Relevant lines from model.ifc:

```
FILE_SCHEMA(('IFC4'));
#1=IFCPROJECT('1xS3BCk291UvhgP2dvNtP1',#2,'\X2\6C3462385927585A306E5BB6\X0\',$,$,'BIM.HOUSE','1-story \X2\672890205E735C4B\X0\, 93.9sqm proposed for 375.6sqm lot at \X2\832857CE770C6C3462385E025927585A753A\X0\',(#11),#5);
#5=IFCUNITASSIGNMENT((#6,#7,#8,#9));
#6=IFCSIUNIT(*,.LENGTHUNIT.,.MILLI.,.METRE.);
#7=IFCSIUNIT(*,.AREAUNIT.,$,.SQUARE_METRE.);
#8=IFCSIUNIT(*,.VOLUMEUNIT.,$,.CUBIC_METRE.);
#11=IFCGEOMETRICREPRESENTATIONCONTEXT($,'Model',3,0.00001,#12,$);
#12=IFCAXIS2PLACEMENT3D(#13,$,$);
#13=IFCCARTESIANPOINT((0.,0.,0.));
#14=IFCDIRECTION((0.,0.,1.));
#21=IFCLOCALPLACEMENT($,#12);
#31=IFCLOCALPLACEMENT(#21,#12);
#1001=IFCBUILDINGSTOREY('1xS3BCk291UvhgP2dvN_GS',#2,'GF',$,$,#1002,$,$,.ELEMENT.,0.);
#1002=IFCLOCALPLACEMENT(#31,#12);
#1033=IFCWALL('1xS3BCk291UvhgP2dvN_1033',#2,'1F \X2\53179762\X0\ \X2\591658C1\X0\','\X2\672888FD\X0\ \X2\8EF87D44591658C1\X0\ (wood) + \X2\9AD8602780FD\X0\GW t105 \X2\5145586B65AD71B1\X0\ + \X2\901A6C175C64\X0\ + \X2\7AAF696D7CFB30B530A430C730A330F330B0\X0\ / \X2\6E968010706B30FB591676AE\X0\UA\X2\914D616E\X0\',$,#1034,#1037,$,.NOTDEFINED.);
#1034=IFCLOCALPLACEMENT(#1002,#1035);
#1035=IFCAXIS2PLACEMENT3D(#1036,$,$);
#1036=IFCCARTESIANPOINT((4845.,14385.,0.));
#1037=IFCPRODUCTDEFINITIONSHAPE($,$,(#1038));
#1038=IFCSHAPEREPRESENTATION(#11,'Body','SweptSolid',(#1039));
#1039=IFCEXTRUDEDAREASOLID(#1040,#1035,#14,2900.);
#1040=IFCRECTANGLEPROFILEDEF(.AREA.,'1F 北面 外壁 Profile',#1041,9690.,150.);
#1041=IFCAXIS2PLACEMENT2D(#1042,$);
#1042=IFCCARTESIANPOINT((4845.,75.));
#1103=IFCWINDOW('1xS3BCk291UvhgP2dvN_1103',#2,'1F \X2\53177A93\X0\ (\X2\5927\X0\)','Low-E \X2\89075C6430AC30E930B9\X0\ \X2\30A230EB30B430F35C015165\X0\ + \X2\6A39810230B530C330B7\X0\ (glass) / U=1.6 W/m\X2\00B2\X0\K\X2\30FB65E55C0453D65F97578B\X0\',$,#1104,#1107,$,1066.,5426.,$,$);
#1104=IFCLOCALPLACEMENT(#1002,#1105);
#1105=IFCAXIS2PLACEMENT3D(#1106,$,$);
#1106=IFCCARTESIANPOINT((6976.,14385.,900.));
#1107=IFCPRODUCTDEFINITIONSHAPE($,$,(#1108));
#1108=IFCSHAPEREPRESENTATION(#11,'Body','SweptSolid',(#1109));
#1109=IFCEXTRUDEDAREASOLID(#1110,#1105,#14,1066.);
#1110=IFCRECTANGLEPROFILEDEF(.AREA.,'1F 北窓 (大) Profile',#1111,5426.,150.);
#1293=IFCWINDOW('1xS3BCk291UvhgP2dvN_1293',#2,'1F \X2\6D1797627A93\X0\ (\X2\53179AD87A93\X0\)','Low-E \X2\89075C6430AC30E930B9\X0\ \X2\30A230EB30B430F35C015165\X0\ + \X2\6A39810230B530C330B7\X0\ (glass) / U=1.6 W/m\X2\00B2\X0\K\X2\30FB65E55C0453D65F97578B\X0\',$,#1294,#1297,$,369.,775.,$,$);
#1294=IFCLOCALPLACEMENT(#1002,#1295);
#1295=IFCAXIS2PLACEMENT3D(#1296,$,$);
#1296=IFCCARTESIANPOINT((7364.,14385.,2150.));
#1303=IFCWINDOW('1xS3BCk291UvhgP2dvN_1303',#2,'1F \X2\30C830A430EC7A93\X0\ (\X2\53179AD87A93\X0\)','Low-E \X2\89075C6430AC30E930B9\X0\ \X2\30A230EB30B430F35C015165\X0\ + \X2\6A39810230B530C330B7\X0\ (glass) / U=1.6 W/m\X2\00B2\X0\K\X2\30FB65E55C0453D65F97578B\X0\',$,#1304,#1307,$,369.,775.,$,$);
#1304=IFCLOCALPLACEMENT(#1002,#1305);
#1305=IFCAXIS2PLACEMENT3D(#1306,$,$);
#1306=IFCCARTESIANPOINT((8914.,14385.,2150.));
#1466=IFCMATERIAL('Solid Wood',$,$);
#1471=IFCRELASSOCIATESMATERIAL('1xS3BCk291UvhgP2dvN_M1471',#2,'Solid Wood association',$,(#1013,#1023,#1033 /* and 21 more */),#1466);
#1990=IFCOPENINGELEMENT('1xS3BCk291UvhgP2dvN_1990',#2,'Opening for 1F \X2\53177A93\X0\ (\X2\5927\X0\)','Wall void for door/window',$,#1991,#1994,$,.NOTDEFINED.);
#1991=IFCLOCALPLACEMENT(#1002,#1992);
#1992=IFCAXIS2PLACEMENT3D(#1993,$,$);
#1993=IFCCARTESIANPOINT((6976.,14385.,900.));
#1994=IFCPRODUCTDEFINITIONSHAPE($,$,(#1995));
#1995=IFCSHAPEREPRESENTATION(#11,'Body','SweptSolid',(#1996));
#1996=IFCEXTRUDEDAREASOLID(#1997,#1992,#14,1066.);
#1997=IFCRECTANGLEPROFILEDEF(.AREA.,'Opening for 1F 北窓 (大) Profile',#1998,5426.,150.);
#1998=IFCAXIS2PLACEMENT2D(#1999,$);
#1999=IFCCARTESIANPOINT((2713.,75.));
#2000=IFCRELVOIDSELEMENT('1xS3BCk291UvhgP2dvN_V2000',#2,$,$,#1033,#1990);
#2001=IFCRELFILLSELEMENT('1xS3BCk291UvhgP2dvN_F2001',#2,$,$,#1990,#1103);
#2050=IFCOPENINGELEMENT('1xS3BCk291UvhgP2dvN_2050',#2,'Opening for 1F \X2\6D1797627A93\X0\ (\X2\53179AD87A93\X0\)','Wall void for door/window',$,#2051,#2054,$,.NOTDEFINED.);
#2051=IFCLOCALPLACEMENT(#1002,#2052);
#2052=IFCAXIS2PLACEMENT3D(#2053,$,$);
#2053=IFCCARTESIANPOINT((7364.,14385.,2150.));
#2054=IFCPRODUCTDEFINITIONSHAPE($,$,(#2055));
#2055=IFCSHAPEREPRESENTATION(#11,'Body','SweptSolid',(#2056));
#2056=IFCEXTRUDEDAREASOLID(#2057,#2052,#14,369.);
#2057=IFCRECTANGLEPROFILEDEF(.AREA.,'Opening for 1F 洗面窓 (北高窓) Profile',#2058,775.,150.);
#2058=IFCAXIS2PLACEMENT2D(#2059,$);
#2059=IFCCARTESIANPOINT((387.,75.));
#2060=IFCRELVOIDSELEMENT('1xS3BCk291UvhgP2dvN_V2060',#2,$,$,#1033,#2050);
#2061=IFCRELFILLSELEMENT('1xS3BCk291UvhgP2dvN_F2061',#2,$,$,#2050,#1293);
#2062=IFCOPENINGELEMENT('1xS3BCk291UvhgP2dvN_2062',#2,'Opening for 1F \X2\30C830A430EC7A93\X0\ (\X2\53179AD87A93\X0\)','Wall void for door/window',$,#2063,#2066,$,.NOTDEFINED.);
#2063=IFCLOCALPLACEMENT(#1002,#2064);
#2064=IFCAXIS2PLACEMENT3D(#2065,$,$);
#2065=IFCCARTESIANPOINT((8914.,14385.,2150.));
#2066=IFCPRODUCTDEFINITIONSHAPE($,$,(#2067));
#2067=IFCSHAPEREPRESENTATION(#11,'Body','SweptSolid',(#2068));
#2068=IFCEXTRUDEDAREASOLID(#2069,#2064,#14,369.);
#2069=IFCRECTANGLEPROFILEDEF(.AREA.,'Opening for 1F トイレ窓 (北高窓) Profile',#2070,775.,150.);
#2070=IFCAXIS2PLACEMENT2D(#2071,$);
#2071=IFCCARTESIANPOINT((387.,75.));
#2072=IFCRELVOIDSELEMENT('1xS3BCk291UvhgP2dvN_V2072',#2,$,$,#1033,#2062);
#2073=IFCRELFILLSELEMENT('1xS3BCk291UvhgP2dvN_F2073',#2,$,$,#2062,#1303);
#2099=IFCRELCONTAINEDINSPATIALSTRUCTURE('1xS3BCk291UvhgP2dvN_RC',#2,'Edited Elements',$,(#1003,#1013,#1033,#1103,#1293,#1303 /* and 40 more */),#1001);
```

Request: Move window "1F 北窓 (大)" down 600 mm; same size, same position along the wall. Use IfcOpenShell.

```python
import numpy as np
import ifcopenshell
import ifcopenshell.api.geometry
import ifcopenshell.util.placement
import ifcopenshell.util.unit

model = ifcopenshell.open("model.ifc")
unit_scale = ifcopenshell.util.unit.calculate_unit_scale(model)

window = model.by_guid("1xS3BCk291UvhgP2dvN_1103")
opening = window.FillsVoids[0].RelatingOpeningElement
dz = -600.0

shift = np.array([0.0, 0.0, dz])
# The window is not placed relative to its opening, so move both.
for product in (opening, window):
    matrix = ifcopenshell.util.placement.get_local_placement(product.ObjectPlacement)
    matrix[:3, 3] += shift
    ifcopenshell.api.geometry.edit_object_placement(model, product=product, matrix=matrix, is_si=False)

print(f"moved by {dz * unit_scale:+.3f} m")

model.write("model_edited.ifc")
```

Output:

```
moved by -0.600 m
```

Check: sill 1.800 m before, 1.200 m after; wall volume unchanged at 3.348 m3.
